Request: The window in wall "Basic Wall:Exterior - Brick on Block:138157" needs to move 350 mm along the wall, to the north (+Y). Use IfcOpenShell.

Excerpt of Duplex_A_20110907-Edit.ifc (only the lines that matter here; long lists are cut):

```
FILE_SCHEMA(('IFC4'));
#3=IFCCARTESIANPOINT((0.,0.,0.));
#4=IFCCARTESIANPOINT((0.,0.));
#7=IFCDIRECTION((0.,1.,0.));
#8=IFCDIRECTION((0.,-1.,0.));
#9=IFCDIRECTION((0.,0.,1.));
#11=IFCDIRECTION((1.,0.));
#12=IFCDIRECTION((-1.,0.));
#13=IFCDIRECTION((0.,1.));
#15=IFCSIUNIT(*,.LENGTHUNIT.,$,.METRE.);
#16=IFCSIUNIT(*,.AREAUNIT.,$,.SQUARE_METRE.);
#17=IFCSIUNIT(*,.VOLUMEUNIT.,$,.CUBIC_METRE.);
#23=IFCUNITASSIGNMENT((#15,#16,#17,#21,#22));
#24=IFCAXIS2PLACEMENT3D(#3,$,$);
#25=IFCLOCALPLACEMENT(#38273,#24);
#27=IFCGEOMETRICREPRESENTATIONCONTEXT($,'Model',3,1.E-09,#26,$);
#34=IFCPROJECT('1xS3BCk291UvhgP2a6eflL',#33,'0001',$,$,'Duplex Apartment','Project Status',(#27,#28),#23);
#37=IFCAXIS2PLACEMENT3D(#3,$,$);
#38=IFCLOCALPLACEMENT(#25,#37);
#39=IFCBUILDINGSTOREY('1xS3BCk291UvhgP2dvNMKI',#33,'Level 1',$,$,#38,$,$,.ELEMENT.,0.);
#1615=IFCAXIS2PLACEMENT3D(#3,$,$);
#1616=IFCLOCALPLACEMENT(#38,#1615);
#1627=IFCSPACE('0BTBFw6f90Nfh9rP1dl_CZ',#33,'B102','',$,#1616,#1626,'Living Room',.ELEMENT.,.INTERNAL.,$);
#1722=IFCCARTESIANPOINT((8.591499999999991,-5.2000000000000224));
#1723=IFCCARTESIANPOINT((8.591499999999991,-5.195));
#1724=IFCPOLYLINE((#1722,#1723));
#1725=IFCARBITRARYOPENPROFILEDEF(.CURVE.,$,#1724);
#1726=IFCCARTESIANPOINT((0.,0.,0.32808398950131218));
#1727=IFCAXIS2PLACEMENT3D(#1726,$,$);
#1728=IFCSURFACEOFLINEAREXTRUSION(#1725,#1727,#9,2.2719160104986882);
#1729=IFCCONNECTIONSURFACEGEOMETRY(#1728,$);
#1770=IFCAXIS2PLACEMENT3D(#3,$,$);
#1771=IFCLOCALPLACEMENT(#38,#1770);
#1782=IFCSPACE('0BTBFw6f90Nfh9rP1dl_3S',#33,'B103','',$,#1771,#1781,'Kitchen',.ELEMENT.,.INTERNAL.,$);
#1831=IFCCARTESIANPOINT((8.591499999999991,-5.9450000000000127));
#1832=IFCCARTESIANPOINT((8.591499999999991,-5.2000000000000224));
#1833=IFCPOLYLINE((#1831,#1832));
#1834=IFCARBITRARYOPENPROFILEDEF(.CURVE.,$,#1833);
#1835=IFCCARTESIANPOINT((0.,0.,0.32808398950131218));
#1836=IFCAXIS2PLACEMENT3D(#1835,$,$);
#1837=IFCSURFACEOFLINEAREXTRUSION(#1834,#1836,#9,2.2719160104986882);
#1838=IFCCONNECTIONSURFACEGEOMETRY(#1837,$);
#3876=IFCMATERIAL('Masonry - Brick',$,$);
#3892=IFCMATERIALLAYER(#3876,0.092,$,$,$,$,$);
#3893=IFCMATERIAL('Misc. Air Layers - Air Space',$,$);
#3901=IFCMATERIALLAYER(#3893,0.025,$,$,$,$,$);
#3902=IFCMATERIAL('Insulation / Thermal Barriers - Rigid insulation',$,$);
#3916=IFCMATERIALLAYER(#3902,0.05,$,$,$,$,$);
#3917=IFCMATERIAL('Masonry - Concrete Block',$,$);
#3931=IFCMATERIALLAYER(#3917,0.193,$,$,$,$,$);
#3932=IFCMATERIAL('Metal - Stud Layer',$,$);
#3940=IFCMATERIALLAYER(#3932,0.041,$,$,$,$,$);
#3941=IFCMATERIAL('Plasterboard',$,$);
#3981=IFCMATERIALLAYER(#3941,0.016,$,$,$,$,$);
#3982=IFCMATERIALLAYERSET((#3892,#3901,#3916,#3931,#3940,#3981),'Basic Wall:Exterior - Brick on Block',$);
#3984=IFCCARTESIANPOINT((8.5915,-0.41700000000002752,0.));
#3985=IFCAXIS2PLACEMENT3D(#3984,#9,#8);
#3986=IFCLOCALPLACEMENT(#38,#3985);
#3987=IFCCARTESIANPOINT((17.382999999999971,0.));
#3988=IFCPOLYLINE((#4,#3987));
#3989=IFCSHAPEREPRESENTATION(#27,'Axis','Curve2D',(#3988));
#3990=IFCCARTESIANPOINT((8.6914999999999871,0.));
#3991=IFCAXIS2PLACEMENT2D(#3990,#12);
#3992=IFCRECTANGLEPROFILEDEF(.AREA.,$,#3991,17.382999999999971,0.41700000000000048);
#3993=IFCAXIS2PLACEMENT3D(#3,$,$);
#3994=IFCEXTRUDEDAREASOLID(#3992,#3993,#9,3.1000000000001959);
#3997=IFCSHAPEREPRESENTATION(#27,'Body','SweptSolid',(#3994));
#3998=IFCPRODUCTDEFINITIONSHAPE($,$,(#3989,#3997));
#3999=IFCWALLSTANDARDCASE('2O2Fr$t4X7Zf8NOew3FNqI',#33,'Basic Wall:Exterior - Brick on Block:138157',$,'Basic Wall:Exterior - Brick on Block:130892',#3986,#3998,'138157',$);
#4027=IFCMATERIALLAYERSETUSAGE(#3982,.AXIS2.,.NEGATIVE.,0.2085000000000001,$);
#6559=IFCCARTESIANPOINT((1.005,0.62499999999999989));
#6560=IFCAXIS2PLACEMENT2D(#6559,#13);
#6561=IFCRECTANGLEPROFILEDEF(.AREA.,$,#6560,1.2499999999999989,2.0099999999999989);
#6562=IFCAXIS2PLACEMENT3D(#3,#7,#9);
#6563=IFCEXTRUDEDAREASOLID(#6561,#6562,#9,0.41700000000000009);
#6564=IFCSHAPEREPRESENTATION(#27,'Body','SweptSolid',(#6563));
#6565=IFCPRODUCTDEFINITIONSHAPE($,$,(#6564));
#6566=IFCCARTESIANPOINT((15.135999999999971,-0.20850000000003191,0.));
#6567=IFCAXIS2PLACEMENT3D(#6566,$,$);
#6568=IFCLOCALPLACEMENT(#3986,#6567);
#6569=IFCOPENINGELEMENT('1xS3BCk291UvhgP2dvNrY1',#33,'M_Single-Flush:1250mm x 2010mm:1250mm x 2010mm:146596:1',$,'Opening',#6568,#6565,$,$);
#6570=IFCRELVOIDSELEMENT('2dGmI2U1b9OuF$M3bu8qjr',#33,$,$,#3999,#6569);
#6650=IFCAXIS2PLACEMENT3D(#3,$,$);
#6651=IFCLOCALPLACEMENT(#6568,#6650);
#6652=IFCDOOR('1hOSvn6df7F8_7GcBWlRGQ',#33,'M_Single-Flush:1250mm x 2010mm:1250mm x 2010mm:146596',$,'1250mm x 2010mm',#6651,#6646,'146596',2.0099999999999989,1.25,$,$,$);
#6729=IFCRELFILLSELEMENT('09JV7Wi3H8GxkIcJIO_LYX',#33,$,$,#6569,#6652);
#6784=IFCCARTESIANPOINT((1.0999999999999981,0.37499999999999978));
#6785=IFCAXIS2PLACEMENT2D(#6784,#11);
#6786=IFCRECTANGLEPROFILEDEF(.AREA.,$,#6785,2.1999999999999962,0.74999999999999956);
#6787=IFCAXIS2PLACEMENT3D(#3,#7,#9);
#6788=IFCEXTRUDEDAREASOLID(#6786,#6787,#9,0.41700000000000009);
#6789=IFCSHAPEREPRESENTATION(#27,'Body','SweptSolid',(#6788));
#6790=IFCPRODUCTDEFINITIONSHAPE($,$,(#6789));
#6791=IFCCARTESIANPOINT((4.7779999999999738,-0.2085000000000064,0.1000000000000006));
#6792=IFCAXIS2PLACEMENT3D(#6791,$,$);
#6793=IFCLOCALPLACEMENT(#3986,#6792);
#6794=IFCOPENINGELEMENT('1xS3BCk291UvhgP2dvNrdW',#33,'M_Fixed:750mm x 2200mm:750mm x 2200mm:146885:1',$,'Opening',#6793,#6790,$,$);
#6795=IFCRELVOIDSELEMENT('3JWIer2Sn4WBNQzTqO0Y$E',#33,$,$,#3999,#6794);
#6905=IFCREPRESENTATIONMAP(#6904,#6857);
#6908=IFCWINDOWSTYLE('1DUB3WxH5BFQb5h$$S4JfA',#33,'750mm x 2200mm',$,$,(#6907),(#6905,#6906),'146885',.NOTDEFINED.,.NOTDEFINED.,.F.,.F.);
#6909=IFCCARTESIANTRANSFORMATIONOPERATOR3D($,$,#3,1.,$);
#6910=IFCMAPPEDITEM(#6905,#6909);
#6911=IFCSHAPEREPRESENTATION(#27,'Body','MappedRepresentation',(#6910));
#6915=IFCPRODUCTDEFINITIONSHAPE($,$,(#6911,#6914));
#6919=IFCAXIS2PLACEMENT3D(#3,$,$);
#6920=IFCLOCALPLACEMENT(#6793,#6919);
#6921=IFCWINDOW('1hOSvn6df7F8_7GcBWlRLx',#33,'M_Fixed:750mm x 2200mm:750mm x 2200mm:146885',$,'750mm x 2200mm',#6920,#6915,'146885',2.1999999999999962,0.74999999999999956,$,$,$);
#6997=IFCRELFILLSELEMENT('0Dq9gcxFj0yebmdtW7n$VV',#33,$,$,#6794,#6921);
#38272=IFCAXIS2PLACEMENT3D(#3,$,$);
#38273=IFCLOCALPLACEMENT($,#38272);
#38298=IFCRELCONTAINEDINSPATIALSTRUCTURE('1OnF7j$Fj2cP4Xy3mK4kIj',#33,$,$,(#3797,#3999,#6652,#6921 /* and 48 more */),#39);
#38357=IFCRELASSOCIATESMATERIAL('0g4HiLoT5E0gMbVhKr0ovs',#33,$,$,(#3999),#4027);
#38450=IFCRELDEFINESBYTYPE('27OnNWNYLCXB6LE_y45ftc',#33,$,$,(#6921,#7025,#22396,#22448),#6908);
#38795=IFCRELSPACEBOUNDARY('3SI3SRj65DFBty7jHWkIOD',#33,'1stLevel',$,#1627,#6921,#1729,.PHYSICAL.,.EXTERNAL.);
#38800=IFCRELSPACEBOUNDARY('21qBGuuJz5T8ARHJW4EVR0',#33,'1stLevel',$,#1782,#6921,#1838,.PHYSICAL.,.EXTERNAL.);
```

```python
import numpy as np
import ifcopenshell
import ifcopenshell.api.geometry
import ifcopenshell.util.placement

model = ifcopenshell.open("Duplex_A_20110907-Edit.ifc")

window = model.by_guid("1hOSvn6df7F8_7GcBWlRLx")
opening = window.FillsVoids[0].RelatingOpeningElement
wall = opening.VoidsElements[0].RelatingBuildingElement

wall_matrix = ifcopenshell.util.placement.get_local_placement(wall.ObjectPlacement)
shift = wall_matrix[:3, 0] * -0.35
before = ifcopenshell.util.placement.get_local_placement(window.ObjectPlacement)[:3, 3].copy()

# The window is placed relative to its opening, so it follows when the opening moves.
matrix = ifcopenshell.util.placement.get_local_placement(opening.ObjectPlacement)
matrix[:3, 3] += shift
ifcopenshell.api.geometry.edit_object_placement(
    model, product=opening, matrix=matrix, is_si=False, should_transform_children=True
)

# Space boundary surfaces are stored in each space's coordinates; move them too.
for rel in window.ProvidesBoundaries:
    if not rel.ConnectionGeometry:
        continue
    surface = rel.ConnectionGeometry.SurfaceOnRelatingElement
    space_matrix = ifcopenshell.util.placement.get_local_placement(rel.RelatingSpace.ObjectPlacement)
    point = np.array(surface.Position.Location.Coordinates) + space_matrix[:3, :3].T @ shift
    surface.Position = model.createIfcAxis2Placement3D(
        model.createIfcCartesianPoint(point.tolist()), surface.Position.Axis, surface.Position.RefDirection
    )

after = ifcopenshell.util.placement.get_local_placement(window.ObjectPlacement)[:3, 3]
print("window moved by", (after - before).round(3) + 0.0)

model.write("Duplex_A_20110907-Edit_rev.ifc")
```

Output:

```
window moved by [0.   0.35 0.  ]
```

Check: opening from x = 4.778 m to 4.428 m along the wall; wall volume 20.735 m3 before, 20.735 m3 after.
